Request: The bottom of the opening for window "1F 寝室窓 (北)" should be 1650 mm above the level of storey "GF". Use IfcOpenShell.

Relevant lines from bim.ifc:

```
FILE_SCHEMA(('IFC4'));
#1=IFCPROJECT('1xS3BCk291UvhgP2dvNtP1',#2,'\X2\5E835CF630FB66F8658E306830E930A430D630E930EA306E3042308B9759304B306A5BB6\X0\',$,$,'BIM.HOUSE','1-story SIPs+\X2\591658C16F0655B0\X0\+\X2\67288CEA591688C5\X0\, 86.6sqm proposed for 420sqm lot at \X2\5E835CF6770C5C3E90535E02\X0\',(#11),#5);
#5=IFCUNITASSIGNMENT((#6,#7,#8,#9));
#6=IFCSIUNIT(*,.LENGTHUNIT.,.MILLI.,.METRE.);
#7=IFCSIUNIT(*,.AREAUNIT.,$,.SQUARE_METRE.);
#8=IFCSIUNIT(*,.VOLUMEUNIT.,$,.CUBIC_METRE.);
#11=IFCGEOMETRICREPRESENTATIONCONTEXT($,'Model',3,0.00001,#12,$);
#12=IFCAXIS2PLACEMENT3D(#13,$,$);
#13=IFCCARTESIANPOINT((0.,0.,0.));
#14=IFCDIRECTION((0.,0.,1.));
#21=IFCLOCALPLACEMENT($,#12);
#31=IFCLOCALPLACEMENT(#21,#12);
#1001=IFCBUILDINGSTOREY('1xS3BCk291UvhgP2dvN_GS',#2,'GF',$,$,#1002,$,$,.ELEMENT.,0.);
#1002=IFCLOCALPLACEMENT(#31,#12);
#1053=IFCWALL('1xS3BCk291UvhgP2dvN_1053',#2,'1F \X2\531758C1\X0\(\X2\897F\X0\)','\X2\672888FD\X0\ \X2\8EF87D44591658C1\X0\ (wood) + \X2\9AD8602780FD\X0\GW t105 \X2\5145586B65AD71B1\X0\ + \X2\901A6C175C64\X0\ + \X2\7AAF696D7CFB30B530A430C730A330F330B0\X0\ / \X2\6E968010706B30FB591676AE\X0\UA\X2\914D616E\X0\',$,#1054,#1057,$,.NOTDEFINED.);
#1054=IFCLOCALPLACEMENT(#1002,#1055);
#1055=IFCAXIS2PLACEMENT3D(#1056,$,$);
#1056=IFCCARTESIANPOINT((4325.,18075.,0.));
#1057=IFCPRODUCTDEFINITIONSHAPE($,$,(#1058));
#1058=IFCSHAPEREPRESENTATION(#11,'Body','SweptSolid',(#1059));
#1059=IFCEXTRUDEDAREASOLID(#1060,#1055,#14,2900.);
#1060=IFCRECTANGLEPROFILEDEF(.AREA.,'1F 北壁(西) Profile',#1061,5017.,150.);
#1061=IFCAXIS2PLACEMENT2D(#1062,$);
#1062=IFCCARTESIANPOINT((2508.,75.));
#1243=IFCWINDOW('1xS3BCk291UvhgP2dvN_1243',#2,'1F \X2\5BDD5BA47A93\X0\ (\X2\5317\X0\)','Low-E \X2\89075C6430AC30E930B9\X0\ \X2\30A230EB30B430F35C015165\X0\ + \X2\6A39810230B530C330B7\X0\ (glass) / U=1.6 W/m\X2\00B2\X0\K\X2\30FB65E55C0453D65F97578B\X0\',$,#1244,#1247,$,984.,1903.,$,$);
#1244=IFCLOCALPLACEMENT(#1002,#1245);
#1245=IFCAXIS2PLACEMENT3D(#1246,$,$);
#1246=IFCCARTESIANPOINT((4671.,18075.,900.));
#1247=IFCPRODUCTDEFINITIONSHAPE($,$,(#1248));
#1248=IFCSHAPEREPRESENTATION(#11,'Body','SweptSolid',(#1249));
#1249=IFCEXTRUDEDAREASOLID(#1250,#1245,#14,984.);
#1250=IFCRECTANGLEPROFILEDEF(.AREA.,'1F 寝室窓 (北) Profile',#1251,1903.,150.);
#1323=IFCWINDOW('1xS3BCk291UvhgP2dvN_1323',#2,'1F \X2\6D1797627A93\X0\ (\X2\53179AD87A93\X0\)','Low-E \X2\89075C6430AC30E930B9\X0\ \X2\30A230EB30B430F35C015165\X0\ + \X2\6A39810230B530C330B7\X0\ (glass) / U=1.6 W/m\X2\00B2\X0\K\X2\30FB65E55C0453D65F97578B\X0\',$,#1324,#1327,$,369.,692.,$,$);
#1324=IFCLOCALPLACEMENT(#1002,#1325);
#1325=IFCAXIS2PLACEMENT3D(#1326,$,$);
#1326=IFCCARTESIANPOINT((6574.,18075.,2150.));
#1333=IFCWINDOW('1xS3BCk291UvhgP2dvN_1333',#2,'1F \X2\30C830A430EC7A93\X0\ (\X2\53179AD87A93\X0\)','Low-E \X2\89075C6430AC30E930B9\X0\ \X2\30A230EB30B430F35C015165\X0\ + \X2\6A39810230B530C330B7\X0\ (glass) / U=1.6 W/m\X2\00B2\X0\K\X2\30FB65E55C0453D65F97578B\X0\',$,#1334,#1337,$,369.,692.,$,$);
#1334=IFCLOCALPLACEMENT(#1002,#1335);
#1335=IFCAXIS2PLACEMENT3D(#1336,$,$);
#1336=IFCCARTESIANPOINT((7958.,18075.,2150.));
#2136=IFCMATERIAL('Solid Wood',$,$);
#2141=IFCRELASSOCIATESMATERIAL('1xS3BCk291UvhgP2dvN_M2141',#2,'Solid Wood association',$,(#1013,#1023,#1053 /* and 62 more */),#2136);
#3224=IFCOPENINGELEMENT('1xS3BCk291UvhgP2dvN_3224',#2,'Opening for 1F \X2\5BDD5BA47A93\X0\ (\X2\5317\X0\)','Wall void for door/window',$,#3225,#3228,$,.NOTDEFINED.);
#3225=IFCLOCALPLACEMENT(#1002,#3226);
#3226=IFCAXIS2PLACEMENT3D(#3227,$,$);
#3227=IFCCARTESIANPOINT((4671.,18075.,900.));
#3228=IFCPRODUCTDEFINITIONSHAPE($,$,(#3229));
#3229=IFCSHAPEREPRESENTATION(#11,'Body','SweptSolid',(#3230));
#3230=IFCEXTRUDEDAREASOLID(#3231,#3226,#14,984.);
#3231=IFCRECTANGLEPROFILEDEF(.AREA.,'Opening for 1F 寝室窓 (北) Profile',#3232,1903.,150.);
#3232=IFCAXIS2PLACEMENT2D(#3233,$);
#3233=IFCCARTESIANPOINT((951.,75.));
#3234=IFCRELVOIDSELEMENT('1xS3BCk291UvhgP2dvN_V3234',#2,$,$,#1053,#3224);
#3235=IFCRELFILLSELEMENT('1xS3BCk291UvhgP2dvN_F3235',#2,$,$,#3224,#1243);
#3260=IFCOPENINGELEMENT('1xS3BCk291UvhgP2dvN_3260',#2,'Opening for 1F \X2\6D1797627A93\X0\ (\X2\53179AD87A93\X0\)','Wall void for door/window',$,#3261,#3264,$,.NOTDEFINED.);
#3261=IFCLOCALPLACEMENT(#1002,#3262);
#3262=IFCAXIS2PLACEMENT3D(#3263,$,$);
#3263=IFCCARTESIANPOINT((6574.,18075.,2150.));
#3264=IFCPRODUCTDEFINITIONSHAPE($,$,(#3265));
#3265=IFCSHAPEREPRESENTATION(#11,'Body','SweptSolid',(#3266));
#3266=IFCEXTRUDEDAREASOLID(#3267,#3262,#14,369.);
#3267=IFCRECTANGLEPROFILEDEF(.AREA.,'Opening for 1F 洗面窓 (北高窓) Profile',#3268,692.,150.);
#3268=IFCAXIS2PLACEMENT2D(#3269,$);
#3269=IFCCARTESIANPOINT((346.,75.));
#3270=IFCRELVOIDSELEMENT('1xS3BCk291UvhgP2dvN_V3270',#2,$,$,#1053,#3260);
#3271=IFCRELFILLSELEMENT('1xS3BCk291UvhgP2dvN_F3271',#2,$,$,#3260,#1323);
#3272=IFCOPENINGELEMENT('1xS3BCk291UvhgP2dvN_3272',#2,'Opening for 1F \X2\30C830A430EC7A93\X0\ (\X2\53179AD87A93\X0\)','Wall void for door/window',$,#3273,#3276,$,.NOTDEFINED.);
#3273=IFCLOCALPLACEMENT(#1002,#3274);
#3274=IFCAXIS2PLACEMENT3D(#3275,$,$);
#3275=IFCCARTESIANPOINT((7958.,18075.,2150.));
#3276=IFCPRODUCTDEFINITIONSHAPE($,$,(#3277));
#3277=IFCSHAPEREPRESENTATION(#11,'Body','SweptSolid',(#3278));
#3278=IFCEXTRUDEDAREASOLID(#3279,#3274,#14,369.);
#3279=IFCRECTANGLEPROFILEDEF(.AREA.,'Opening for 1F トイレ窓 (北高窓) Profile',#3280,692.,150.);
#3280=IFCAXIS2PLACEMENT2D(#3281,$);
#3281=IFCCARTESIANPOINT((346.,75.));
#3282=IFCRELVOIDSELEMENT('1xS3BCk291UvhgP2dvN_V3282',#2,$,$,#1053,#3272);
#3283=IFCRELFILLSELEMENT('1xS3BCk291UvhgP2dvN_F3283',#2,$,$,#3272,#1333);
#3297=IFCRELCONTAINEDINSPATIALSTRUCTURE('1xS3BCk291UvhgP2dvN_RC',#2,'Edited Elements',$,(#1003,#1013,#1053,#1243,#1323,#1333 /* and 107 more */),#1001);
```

```python
import numpy as np
import ifcopenshell
import ifcopenshell.api.geometry
import ifcopenshell.geom
import ifcopenshell.util.element
import ifcopenshell.util.placement
import ifcopenshell.util.shape
import ifcopenshell.util.unit

model = ifcopenshell.open("bim.ifc")
unit_scale = ifcopenshell.util.unit.calculate_unit_scale(model)

window = model.by_id(1243)
opening = window.FillsVoids[0].RelatingOpeningElement
storey = ifcopenshell.util.element.get_container(window, ifc_class="IfcBuildingStorey")
level = ifcopenshell.util.placement.get_local_placement(storey.ObjectPlacement)[2, 3]

# The opening's origin need not be at the sill, so measure its lowest point.
shape = ifcopenshell.geom.create_shape(ifcopenshell.geom.settings(), opening)
bottom = ifcopenshell.util.shape.get_shape_bottom_elevation(shape, shape.geometry) / unit_scale
dz = level + 1.65 / unit_scale - bottom

shift = np.array([0.0, 0.0, dz])
# The window is not placed relative to its opening, so move both.
for product in (opening, window):
    matrix = ifcopenshell.util.placement.get_local_placement(product.ObjectPlacement)
    matrix[:3, 3] += shift
    ifcopenshell.api.geometry.edit_object_placement(model, product=product, matrix=matrix, is_si=False)

print(f"moved by {dz * unit_scale:+.3f} m")

model.write("bim-out.ifc")
```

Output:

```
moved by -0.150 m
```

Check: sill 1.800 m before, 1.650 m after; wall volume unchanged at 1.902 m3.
